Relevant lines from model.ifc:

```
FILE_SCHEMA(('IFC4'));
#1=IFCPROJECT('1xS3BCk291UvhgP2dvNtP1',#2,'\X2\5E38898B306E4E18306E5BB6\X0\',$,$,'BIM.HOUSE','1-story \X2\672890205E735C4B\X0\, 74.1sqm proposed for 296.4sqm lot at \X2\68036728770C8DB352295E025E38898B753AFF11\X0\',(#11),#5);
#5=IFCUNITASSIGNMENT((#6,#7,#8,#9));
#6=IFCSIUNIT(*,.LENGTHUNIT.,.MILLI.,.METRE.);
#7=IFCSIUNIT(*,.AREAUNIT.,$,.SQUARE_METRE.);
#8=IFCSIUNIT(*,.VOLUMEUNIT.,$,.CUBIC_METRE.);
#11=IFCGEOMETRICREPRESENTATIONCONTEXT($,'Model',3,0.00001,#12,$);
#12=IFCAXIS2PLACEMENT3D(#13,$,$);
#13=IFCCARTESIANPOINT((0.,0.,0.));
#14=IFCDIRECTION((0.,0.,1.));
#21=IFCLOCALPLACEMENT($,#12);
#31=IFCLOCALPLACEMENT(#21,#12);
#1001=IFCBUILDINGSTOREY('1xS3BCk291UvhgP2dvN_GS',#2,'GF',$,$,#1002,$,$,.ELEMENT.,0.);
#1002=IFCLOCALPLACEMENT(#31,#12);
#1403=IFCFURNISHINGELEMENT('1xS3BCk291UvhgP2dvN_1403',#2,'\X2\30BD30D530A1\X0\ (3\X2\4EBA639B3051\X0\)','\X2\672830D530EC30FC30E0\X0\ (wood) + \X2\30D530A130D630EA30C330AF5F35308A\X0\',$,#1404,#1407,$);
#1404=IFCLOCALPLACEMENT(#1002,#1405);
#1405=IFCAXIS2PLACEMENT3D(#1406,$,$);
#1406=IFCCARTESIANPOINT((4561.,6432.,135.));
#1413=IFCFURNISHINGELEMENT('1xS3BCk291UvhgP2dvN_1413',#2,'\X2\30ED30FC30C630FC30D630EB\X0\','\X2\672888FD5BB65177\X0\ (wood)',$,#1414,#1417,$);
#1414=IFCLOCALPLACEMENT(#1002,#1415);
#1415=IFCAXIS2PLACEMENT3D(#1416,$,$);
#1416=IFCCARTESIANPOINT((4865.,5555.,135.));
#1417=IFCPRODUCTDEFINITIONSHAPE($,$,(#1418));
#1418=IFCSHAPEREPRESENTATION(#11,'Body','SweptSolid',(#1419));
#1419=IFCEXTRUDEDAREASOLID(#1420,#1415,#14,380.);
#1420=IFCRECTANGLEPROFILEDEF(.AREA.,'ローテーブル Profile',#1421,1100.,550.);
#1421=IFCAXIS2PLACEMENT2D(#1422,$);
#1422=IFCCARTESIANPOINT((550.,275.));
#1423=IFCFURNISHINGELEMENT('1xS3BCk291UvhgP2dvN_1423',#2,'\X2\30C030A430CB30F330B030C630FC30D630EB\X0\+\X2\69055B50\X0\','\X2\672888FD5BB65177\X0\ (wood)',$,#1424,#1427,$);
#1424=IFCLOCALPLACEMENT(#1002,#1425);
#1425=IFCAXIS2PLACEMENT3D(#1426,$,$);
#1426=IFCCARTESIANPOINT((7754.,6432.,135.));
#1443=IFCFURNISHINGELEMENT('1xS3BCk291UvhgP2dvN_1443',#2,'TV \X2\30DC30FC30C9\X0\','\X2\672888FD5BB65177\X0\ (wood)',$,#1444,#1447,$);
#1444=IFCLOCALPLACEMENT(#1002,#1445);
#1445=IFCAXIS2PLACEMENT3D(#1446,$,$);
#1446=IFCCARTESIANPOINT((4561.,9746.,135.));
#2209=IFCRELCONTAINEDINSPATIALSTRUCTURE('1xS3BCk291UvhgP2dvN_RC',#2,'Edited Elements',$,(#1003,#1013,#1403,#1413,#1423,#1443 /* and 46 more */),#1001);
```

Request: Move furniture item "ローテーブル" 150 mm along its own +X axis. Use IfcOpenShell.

```python
import ifcopenshell
import ifcopenshell.api.geometry
import ifcopenshell.util.placement
import ifcopenshell.util.unit

model = ifcopenshell.open("model.ifc")
unit_scale = ifcopenshell.util.unit.calculate_unit_scale(model)

item = model.by_guid("1xS3BCk291UvhgP2dvN_1413")
matrix = ifcopenshell.util.placement.get_local_placement(item.ObjectPlacement)
matrix[:3, 3] += matrix[:3, 0] * 0.15 / unit_scale
ifcopenshell.api.geometry.edit_object_placement(model, product=item, matrix=matrix, is_si=False)

print(ifcopenshell.util.placement.get_local_placement(item.ObjectPlacement).round(3) + 0.0)

model.write("model-out.ifc")
```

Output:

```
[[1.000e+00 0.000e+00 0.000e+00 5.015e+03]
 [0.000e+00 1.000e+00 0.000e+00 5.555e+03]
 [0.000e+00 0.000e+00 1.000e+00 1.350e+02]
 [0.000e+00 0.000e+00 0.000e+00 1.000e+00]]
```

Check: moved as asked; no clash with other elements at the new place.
